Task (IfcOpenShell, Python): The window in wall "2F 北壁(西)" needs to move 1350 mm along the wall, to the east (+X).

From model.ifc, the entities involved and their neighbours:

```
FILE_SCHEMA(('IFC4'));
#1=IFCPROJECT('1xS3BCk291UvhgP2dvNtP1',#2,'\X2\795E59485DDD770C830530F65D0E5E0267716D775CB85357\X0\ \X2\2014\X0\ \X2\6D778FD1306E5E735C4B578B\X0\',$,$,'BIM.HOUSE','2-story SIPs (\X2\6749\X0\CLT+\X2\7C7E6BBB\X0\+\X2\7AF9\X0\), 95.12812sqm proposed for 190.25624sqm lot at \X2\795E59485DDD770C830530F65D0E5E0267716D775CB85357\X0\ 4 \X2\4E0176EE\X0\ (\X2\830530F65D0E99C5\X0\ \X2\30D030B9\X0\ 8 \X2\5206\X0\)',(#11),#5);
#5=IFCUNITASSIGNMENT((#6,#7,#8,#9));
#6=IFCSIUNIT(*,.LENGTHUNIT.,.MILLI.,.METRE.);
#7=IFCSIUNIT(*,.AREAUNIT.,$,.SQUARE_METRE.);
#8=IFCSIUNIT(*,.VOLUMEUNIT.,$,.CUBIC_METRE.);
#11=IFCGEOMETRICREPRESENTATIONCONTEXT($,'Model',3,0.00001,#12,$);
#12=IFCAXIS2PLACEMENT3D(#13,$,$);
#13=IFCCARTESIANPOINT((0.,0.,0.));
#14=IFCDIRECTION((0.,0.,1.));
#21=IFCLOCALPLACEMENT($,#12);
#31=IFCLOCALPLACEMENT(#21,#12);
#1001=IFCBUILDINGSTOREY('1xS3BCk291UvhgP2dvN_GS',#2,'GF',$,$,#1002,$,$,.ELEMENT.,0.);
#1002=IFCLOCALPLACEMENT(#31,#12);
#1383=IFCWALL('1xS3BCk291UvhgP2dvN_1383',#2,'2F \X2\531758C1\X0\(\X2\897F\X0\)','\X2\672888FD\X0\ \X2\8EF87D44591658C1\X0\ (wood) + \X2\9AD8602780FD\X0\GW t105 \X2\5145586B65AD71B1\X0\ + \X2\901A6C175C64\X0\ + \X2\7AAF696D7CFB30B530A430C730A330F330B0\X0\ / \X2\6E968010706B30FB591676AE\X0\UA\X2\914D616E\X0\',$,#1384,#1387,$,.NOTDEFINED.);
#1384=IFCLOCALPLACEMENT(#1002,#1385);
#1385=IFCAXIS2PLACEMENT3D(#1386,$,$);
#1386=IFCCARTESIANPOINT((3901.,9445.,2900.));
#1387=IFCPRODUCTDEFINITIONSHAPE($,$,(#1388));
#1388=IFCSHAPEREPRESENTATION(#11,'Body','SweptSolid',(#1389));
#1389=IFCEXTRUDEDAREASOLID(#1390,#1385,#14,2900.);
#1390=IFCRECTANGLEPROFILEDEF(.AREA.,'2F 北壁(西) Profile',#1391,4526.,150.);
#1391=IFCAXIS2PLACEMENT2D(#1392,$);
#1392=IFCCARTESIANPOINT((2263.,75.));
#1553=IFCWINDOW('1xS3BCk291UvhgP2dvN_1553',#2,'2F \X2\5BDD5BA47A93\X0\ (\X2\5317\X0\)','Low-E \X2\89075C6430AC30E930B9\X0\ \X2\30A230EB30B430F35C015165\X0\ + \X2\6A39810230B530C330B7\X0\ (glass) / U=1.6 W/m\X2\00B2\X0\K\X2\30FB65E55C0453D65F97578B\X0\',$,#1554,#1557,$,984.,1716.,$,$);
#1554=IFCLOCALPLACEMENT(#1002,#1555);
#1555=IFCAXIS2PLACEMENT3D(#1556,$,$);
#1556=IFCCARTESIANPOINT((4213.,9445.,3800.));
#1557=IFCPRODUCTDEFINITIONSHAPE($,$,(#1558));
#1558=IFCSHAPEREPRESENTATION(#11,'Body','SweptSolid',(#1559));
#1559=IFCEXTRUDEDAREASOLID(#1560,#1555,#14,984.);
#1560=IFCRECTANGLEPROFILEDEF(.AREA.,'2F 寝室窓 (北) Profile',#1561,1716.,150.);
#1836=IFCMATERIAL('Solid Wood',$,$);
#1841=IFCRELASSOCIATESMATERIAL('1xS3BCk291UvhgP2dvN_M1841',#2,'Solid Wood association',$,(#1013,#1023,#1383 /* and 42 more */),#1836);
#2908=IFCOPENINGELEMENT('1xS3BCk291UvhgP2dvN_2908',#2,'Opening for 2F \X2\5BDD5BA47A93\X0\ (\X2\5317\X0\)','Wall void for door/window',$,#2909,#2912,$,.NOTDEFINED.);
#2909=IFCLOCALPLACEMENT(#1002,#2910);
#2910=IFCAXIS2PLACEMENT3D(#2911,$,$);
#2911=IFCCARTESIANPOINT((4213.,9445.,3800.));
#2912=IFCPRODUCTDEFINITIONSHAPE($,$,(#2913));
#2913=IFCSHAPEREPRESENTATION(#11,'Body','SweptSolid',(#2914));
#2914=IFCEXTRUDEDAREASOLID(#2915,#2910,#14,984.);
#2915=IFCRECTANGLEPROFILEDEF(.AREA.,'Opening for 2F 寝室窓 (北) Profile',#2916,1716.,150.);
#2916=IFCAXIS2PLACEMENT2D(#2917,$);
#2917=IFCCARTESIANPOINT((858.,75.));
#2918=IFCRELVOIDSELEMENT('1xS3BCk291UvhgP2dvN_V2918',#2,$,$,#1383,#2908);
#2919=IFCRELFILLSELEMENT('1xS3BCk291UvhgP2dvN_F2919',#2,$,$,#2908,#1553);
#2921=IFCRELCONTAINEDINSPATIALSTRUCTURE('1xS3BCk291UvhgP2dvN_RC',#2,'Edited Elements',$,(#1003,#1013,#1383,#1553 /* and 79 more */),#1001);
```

```python
import ifcopenshell
import ifcopenshell.api.geometry
import ifcopenshell.util.placement
import ifcopenshell.util.unit

model = ifcopenshell.open("model.ifc")
unit_scale = ifcopenshell.util.unit.calculate_unit_scale(model)

window = model.by_guid("1xS3BCk291UvhgP2dvN_1553")
opening = window.FillsVoids[0].RelatingOpeningElement
wall = opening.VoidsElements[0].RelatingBuildingElement

wall_matrix = ifcopenshell.util.placement.get_local_placement(wall.ObjectPlacement)
shift = wall_matrix[:3, 0] * 1.35 / unit_scale
before = ifcopenshell.util.placement.get_local_placement(window.ObjectPlacement)[:3, 3].copy()

# The window is not placed relative to its opening, so move both.
for product in (opening, window):
    matrix = ifcopenshell.util.placement.get_local_placement(product.ObjectPlacement)
    matrix[:3, 3] += shift
    ifcopenshell.api.geometry.edit_object_placement(model, product=product, matrix=matrix, is_si=False)

after = ifcopenshell.util.placement.get_local_placement(window.ObjectPlacement)[:3, 3]
print("window moved by", (after - before).round(3) + 0.0)

model.write("model_edited.ifc")
```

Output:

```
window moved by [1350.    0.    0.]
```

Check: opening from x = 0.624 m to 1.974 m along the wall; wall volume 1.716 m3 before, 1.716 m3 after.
